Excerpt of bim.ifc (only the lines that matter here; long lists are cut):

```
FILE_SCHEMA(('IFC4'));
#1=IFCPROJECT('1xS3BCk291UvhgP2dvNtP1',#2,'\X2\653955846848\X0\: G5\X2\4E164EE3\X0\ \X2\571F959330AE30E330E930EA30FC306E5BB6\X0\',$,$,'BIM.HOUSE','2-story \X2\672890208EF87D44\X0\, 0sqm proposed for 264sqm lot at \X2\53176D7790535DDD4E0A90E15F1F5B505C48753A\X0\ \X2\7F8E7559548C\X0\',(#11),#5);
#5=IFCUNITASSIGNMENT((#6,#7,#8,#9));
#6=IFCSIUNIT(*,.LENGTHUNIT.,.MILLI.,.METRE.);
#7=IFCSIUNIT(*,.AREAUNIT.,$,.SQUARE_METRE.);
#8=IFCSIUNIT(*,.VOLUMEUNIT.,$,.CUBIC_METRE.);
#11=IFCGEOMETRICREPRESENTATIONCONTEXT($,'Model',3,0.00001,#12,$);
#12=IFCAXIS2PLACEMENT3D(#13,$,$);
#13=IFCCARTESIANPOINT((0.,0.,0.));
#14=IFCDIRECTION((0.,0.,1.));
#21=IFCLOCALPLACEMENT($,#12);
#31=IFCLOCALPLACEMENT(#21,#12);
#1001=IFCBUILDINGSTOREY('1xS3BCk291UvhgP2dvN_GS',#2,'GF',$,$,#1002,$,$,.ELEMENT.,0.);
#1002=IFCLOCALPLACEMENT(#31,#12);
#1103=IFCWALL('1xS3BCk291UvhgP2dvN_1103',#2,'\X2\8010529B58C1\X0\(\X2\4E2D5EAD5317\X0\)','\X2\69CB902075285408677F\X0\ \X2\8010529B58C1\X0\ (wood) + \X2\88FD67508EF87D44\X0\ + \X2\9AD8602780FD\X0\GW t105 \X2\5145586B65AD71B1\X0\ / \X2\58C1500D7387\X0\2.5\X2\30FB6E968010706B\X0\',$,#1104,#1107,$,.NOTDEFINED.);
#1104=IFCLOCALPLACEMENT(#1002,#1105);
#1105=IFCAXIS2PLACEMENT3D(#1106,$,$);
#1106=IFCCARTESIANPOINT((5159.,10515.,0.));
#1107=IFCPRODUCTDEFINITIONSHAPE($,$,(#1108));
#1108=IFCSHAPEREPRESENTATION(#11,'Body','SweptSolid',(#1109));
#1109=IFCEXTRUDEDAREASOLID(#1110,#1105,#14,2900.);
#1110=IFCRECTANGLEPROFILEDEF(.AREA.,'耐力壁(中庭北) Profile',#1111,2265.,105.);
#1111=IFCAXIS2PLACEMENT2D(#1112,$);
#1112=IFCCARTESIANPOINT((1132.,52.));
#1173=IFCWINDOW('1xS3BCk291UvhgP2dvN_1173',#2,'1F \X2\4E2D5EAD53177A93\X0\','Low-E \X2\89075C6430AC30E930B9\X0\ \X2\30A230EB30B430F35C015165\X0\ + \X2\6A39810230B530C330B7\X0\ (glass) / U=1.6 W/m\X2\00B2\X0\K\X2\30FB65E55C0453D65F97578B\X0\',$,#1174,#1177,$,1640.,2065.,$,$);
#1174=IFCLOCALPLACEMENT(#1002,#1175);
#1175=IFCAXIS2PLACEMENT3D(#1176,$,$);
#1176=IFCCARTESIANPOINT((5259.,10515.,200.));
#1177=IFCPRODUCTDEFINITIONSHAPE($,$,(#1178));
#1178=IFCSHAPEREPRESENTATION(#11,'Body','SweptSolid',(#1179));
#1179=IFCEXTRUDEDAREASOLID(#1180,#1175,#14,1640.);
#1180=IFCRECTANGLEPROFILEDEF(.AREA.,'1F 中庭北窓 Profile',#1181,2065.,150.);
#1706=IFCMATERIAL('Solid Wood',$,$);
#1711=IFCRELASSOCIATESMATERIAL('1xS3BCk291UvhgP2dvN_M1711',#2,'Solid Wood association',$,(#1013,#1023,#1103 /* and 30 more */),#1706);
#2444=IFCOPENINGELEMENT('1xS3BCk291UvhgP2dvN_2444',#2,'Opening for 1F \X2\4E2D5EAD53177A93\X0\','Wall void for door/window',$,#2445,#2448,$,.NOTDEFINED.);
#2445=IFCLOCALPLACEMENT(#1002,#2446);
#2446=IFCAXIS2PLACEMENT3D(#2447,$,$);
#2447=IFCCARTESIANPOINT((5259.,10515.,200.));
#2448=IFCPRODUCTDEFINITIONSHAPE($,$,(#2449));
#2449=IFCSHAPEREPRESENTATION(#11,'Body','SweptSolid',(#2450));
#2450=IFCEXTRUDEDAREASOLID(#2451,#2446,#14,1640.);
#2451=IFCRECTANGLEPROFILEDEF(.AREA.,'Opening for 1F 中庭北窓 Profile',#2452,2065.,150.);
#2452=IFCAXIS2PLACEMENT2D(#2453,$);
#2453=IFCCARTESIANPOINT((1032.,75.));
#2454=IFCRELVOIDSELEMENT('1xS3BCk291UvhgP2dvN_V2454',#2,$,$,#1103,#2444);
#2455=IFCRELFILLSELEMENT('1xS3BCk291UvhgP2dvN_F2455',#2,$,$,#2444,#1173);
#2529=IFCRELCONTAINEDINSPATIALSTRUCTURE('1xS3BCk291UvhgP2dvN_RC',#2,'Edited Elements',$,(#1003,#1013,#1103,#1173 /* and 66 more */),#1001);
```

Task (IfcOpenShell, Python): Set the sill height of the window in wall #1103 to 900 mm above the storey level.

```python
import numpy as np
import ifcopenshell
import ifcopenshell.api.geometry
import ifcopenshell.geom
import ifcopenshell.util.element
import ifcopenshell.util.placement
import ifcopenshell.util.shape
import ifcopenshell.util.unit

model = ifcopenshell.open("bim.ifc")
unit_scale = ifcopenshell.util.unit.calculate_unit_scale(model)

window = model.by_id(1173)
opening = window.FillsVoids[0].RelatingOpeningElement
storey = ifcopenshell.util.element.get_container(window, ifc_class="IfcBuildingStorey")
level = ifcopenshell.util.placement.get_local_placement(storey.ObjectPlacement)[2, 3]

# The opening's origin need not be at the sill, so measure its lowest point.
shape = ifcopenshell.geom.create_shape(ifcopenshell.geom.settings(), opening)
bottom = ifcopenshell.util.shape.get_shape_bottom_elevation(shape, shape.geometry) / unit_scale
dz = level + 0.9 / unit_scale - bottom

shift = np.array([0.0, 0.0, dz])
# The window is not placed relative to its opening, so move both.
for product in (opening, window):
    matrix = ifcopenshell.util.placement.get_local_placement(product.ObjectPlacement)
    matrix[:3, 3] += shift
    ifcopenshell.api.geometry.edit_object_placement(model, product=product, matrix=matrix, is_si=False)

print(f"moved by {dz * unit_scale:+.3f} m")

model.write("bim_edited.ifc")
```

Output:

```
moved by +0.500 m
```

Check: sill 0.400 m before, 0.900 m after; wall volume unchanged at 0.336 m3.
